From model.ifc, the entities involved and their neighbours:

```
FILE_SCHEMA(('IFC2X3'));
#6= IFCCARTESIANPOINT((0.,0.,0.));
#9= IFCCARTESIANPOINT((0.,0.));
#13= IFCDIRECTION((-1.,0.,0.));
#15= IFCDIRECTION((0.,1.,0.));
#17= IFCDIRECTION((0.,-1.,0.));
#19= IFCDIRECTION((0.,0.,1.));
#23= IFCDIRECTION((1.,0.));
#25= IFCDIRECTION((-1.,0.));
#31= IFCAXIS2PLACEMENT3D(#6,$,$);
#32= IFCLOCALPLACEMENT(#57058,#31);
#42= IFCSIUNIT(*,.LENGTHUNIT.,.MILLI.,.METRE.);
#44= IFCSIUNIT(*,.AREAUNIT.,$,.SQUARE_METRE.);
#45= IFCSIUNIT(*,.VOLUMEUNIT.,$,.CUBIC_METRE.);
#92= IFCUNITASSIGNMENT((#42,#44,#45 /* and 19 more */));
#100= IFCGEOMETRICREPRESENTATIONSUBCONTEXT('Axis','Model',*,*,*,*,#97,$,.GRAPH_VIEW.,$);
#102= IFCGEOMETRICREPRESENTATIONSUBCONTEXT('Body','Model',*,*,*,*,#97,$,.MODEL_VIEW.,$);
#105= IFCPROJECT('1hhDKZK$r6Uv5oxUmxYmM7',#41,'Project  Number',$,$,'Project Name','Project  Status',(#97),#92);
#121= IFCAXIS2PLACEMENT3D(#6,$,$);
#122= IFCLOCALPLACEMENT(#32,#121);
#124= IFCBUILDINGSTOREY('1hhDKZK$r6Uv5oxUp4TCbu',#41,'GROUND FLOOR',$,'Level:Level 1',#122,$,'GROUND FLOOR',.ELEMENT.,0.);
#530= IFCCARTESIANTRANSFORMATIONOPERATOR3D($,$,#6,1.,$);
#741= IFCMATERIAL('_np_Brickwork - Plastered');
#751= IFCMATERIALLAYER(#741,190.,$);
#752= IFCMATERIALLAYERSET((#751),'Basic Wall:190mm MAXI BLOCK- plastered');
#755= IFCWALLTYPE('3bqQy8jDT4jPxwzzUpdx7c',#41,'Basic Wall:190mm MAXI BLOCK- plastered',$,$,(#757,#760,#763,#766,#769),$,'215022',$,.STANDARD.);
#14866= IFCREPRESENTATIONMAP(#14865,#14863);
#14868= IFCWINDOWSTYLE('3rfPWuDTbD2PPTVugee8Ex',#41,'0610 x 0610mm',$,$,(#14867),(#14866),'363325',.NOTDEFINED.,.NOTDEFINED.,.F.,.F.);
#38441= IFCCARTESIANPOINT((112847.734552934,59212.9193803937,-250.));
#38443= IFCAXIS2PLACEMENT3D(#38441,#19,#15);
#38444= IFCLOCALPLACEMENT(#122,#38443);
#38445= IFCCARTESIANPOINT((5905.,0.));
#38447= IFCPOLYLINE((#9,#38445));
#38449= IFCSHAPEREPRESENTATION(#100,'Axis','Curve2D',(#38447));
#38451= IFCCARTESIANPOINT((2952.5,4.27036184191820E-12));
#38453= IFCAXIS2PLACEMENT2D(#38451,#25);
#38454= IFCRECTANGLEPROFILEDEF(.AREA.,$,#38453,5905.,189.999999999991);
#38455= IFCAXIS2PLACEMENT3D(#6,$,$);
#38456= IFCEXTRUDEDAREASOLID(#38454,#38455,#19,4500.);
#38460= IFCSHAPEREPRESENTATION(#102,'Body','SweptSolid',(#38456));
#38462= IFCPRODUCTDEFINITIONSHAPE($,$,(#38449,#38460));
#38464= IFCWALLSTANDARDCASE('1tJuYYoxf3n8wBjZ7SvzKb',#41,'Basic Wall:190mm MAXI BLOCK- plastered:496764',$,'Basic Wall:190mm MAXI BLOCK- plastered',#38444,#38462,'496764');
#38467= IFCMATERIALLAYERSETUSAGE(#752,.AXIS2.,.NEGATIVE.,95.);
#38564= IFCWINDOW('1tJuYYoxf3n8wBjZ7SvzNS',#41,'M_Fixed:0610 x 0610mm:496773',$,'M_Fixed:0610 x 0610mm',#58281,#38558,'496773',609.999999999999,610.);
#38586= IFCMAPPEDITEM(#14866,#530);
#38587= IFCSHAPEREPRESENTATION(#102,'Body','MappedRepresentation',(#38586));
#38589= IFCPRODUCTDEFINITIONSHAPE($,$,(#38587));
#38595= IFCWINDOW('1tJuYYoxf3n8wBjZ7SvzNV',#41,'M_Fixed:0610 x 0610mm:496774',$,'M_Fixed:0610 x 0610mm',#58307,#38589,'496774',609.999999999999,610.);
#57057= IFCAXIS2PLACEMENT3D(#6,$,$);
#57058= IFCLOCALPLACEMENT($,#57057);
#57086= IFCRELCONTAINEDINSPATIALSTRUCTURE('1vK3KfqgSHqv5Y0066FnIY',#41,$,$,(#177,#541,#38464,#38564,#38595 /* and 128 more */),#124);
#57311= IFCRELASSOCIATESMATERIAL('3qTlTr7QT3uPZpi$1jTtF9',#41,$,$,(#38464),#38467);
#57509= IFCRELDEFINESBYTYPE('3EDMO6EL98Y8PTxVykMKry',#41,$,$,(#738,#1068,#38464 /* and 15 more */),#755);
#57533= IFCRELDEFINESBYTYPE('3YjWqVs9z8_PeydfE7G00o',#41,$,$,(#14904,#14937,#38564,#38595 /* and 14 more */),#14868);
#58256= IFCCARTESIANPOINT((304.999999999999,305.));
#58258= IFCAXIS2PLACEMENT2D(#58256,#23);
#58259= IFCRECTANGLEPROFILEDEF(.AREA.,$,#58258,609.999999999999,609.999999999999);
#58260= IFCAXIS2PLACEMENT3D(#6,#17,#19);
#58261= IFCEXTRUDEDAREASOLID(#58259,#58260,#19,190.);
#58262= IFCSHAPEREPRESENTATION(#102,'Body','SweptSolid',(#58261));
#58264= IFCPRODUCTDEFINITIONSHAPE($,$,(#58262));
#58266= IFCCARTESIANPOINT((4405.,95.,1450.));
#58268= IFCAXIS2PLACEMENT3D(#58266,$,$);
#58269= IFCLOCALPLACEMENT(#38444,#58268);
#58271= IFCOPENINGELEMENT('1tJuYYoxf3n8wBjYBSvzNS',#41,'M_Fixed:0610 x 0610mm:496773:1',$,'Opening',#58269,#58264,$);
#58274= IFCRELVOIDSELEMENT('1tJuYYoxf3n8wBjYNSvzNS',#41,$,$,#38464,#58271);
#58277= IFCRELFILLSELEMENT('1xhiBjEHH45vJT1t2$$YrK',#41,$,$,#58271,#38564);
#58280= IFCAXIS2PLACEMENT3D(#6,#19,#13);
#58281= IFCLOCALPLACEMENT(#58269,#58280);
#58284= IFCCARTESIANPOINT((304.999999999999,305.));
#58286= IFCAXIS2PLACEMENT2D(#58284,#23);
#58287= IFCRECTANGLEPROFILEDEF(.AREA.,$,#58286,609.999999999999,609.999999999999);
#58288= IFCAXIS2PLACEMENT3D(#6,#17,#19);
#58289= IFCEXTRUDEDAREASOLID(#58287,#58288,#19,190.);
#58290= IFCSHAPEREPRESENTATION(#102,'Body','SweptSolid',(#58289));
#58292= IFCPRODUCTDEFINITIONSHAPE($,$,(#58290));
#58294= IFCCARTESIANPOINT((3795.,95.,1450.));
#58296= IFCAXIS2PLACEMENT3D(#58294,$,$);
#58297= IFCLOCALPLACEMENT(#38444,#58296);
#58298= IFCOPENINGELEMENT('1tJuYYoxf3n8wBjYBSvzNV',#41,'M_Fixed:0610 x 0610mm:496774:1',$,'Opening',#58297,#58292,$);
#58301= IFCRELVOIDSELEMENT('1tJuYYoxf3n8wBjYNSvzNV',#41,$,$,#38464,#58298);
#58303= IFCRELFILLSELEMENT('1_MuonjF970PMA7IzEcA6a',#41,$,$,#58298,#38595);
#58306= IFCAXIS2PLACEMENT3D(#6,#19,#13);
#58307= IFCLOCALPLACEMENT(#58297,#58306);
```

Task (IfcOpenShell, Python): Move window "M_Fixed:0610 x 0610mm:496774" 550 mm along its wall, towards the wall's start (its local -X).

```python
import ifcopenshell
import ifcopenshell.api.geometry
import ifcopenshell.util.placement
import ifcopenshell.util.unit

model = ifcopenshell.open("model.ifc")
unit_scale = ifcopenshell.util.unit.calculate_unit_scale(model)

window = model.by_guid("1tJuYYoxf3n8wBjZ7SvzNV")
opening = window.FillsVoids[0].RelatingOpeningElement
wall = opening.VoidsElements[0].RelatingBuildingElement

wall_matrix = ifcopenshell.util.placement.get_local_placement(wall.ObjectPlacement)
shift = wall_matrix[:3, 0] * -0.55 / unit_scale
before = ifcopenshell.util.placement.get_local_placement(window.ObjectPlacement)[:3, 3].copy()

# The window is placed relative to its opening, so it follows when the opening moves.
matrix = ifcopenshell.util.placement.get_local_placement(opening.ObjectPlacement)
matrix[:3, 3] += shift
ifcopenshell.api.geometry.edit_object_placement(
    model, product=opening, matrix=matrix, is_si=False, should_transform_children=True
)

after = ifcopenshell.util.placement.get_local_placement(window.ObjectPlacement)[:3, 3]
print("window moved by", (after - before).round(3) + 0.0)

model.write("model_rev.ifc")
```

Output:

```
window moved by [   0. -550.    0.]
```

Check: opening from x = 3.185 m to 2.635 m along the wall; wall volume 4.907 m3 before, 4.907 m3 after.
